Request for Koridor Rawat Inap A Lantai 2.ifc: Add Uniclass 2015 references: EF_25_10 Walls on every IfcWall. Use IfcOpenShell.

First a look at what the model holds.

```python
import ifcopenshell

model = ifcopenshell.open("Koridor Rawat Inap A Lantai 2.ifc")
print(model.schema)
print("classifications:", [c.Name for c in model.by_type("IfcClassification")])
for ifc_class in ("IfcDoor", "IfcRoof", "IfcStair", "IfcWall", "IfcWindow"):
    print(ifc_class, len(model.by_type(ifc_class)))
```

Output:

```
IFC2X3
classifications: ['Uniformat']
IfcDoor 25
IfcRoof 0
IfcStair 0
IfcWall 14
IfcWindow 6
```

```python
import ifcopenshell
import ifcopenshell.api.classification

model = ifcopenshell.open("Koridor Rawat Inap A Lantai 2.ifc")

# IFC2X3 requires Source and Edition and has no link from the project to the system.
system = model.create_entity("IfcClassification", Source="NBS", Edition="2015", Name="Uniclass 2015")

codes = {
    "IfcWall": ("EF_25_10", "Walls"),
}
for ifc_class, (code, name) in codes.items():
    products = model.by_type(ifc_class)
    ifcopenshell.api.classification.add_reference(
        model, products=products, classification=system, identification=code, name=name
    )
    print(code, len(products))

model.write("Koridor Rawat Inap A Lantai 2_edited.ifc")
```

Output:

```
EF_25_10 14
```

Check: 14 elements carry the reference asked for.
